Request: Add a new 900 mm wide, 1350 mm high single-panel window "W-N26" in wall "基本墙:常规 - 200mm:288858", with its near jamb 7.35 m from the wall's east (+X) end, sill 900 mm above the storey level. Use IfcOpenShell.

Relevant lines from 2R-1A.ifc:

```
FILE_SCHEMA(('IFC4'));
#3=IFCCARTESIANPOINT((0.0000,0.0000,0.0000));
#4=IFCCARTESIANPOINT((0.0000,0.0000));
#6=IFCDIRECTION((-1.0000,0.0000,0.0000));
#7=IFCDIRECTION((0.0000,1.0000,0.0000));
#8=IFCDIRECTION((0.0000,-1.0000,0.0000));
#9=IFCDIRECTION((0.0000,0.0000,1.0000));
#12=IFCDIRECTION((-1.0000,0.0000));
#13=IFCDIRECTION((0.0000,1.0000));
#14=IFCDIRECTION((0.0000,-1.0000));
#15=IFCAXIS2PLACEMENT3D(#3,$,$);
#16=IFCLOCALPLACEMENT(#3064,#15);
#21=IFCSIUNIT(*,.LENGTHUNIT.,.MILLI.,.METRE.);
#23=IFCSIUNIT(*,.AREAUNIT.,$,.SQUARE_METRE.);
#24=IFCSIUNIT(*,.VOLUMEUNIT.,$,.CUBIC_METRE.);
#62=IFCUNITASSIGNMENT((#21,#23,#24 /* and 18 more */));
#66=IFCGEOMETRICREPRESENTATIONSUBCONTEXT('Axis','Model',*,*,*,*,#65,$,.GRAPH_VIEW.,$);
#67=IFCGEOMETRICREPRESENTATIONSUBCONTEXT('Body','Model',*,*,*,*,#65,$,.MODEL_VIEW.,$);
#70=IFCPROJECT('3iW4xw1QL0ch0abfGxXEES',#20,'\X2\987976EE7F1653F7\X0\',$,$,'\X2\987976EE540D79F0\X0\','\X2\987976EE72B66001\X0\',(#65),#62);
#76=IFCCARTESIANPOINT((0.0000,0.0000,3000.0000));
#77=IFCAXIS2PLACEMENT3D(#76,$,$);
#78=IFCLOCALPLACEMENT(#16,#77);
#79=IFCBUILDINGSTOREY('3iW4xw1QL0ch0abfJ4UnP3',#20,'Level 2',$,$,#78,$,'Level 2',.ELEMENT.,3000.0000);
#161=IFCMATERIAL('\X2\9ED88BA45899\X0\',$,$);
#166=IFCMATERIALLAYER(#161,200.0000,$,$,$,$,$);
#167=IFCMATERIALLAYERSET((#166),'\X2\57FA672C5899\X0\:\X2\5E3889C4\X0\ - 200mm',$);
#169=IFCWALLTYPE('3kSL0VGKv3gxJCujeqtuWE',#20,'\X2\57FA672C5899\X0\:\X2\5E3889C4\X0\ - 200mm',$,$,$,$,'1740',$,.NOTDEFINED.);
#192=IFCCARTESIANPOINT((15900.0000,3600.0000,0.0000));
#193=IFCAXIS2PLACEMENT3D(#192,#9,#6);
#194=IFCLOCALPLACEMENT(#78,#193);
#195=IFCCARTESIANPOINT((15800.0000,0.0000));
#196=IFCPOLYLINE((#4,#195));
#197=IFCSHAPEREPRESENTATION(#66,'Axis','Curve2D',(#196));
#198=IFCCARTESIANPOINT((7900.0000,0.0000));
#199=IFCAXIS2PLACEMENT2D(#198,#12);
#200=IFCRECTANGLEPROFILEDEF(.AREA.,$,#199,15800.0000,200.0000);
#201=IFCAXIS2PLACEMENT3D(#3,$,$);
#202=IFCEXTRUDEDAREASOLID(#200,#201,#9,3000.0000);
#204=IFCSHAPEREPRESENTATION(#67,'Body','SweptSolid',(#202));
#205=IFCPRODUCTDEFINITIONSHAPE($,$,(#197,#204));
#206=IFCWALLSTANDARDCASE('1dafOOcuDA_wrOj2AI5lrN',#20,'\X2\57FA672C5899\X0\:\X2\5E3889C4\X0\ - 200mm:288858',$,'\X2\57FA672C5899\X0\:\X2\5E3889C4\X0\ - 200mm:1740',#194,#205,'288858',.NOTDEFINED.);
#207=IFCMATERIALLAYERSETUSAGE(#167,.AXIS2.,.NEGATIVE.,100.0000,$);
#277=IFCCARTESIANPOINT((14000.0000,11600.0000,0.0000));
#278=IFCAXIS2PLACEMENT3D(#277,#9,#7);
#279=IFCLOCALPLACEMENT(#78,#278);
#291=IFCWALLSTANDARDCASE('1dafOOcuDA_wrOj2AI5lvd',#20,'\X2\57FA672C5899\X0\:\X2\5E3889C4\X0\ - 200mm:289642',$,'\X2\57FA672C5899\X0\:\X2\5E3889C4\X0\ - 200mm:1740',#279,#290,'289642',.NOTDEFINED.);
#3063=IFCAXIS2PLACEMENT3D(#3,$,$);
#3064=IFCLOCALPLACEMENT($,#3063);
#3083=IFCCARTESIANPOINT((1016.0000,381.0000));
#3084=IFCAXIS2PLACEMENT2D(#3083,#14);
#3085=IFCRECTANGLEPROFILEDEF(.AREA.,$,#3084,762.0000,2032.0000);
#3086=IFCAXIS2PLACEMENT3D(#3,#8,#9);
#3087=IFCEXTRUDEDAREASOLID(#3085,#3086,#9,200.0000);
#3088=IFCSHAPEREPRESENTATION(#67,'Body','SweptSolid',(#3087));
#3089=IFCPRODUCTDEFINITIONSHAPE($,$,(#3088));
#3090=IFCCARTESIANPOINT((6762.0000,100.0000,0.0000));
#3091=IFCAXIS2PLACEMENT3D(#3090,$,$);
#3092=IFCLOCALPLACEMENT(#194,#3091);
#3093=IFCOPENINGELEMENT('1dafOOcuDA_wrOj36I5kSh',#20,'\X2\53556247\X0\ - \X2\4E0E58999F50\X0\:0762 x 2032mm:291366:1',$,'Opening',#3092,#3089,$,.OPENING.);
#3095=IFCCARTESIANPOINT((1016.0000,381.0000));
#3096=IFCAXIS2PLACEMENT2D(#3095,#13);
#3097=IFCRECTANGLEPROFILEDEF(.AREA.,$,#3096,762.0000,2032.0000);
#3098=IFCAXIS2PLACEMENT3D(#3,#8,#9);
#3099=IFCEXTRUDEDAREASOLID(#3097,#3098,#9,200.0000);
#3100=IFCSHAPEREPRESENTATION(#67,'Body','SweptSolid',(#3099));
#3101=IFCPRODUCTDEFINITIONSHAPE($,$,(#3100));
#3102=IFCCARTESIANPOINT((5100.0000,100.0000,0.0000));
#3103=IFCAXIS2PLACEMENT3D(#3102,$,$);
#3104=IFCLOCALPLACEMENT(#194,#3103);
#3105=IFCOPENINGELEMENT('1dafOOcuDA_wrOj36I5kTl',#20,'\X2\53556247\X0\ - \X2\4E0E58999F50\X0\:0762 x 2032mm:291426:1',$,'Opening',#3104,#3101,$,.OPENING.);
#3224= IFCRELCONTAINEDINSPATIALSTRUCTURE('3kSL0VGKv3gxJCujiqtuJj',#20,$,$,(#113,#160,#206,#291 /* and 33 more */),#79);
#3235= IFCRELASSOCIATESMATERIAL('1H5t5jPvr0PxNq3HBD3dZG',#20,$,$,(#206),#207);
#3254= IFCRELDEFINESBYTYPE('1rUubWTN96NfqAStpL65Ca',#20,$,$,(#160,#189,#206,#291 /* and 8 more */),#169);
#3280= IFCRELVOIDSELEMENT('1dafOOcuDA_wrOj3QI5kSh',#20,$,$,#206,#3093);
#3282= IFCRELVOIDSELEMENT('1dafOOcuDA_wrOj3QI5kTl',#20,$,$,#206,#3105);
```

```python
import numpy as np
import ifcopenshell
import ifcopenshell.api.feature
import ifcopenshell.api.geometry
import ifcopenshell.api.root
import ifcopenshell.api.spatial
import ifcopenshell.geom
import ifcopenshell.util.element
import ifcopenshell.util.placement
import ifcopenshell.util.representation
import ifcopenshell.util.shape
import ifcopenshell.util.unit

model = ifcopenshell.open("2R-1A.ifc")
unit_scale = ifcopenshell.util.unit.calculate_unit_scale(model)
settings = ifcopenshell.geom.settings()


def volume(element):
    """Net volume in cubic metres, openings subtracted."""
    shape = ifcopenshell.geom.create_shape(settings, element)
    return ifcopenshell.util.shape.get_volume(shape.geometry)


wall = model.by_id(206)
storey = ifcopenshell.util.element.get_container(wall, ifc_class="IfcBuildingStorey")
context = ifcopenshell.util.representation.get_context(model, "Model", "Body", "MODEL_VIEW")
before = volume(wall)

width, height, from_end, sill = 0.9, 1.35, 7.35, 0.9  # metres

# The wall runs along its own X axis, and the end named is its -X end.
wall_shape = ifcopenshell.geom.create_shape(settings, wall)
x, y, z = ifcopenshell.util.shape.get_vertices(wall_shape.geometry).T
start = x.min() + from_end
face, thickness = float(y.min()), float(y.max() - y.min())
wall_matrix = ifcopenshell.util.placement.get_local_placement(wall.ObjectPlacement)
level = ifcopenshell.util.placement.get_local_placement(storey.ObjectPlacement)[2, 3]


def in_wall(x, y):
    """Placement at x, y metres in the wall's axes, at sill height."""
    matrix = wall_matrix.copy()
    matrix[:, 3] = wall_matrix @ np.array([x / unit_scale, y / unit_scale, 0.0, 1.0])
    matrix[2, 3] = level + sill / unit_scale
    return matrix


# Opening: a box that overshoots both wall faces by 50 mm.
opening = ifcopenshell.api.root.create_entity(model, ifc_class="IfcOpeningElement", predefined_type="OPENING")
box = ifcopenshell.api.geometry.add_wall_representation(
    model, context=context, length=width, height=height, thickness=thickness + 0.1
)
ifcopenshell.api.geometry.assign_representation(model, product=opening, representation=box)
ifcopenshell.api.geometry.edit_object_placement(model, product=opening, matrix=in_wall(start, face - 0.05), is_si=False)
ifcopenshell.api.feature.add_feature(model, feature=opening, element=wall)

window = ifcopenshell.api.root.create_entity(model, ifc_class="IfcWindow", name="W-N26", predefined_type="WINDOW")
window.OverallWidth, window.OverallHeight = width / unit_scale, height / unit_scale
window.PartitioningType = "SINGLE_PANEL"
body = ifcopenshell.api.geometry.add_window_representation(
    model,
    context=context,
    overall_width=window.OverallWidth,
    overall_height=window.OverallHeight,
    partition_type="SINGLE_PANEL",
)
ifcopenshell.api.geometry.assign_representation(model, product=window, representation=body)
ifcopenshell.api.spatial.assign_container(model, products=[window], relating_structure=storey)
ifcopenshell.api.feature.add_filling(model, opening=opening, element=window)

# Centre the window in the wall's thickness.
ifcopenshell.api.geometry.edit_object_placement(model, product=window, matrix=in_wall(start, face), is_si=False)
window_shape = ifcopenshell.geom.create_shape(settings, window)
depth = ifcopenshell.util.shape.get_vertices(window_shape.geometry)[:, 1]
offset = face + thickness / 2 - (depth.min() + depth.max()) / 2
ifcopenshell.api.geometry.edit_object_placement(model, product=window, matrix=in_wall(start, offset), is_si=False)

after = volume(wall)

print(f"wall volume {before:.3f} -> {after:.3f} m3")

model.write("2R-1A_rev.ifc")
```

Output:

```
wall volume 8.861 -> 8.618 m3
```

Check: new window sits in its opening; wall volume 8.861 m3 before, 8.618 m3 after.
